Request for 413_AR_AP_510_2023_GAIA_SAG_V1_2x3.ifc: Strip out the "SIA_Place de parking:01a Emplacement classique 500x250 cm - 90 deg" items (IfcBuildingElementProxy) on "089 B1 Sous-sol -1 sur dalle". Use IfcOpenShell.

First a look at what the model holds.

```python
import ifcopenshell
import ifcopenshell.util.element

model = ifcopenshell.open("413_AR_AP_510_2023_GAIA_SAG_V1_2x3.ifc")
print(model.schema)
storey = next(s for s in model.by_type("IfcBuildingStorey") if s.Name == "089 B1 Sous-sol -1 sur dalle")
proxies = [e for e in ifcopenshell.util.element.get_decomposition(storey) if e.is_a("IfcBuildingElementProxy")]
seen = {}
for e in proxies:
    element_type = ifcopenshell.util.element.get_type(e)
    name = element_type.Name if element_type not in (None, e) else None
    seen[name] = seen.get(name, 0) + 1
for name, count in sorted(seen.items(), key=str):
    print(count, "x", name)
```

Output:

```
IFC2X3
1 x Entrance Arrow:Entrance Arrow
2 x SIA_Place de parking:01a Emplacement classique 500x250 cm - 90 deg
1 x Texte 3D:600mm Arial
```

```python
import ifcopenshell
import ifcopenshell.api.root
import ifcopenshell.util.element

model = ifcopenshell.open("413_AR_AP_510_2023_GAIA_SAG_V1_2x3.ifc")

storey = next(s for s in model.by_type("IfcBuildingStorey") if s.Name == "089 B1 Sous-sol -1 sur dalle")
proxies = [e for e in ifcopenshell.util.element.get_decomposition(storey) if e.is_a("IfcBuildingElementProxy")]
targets = [e for e in proxies if (t := ifcopenshell.util.element.get_type(e)) not in (None, e) and t.Name == "SIA_Place de parking:01a Emplacement classique 500x250 cm - 90 deg"]

for e in targets:
    ifcopenshell.api.root.remove_product(model, product=e)
print(len(targets), "removed")

model.write("413_AR_AP_510_2023_GAIA_SAG_V1_2x3_rev.ifc")
```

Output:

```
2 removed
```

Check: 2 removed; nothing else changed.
